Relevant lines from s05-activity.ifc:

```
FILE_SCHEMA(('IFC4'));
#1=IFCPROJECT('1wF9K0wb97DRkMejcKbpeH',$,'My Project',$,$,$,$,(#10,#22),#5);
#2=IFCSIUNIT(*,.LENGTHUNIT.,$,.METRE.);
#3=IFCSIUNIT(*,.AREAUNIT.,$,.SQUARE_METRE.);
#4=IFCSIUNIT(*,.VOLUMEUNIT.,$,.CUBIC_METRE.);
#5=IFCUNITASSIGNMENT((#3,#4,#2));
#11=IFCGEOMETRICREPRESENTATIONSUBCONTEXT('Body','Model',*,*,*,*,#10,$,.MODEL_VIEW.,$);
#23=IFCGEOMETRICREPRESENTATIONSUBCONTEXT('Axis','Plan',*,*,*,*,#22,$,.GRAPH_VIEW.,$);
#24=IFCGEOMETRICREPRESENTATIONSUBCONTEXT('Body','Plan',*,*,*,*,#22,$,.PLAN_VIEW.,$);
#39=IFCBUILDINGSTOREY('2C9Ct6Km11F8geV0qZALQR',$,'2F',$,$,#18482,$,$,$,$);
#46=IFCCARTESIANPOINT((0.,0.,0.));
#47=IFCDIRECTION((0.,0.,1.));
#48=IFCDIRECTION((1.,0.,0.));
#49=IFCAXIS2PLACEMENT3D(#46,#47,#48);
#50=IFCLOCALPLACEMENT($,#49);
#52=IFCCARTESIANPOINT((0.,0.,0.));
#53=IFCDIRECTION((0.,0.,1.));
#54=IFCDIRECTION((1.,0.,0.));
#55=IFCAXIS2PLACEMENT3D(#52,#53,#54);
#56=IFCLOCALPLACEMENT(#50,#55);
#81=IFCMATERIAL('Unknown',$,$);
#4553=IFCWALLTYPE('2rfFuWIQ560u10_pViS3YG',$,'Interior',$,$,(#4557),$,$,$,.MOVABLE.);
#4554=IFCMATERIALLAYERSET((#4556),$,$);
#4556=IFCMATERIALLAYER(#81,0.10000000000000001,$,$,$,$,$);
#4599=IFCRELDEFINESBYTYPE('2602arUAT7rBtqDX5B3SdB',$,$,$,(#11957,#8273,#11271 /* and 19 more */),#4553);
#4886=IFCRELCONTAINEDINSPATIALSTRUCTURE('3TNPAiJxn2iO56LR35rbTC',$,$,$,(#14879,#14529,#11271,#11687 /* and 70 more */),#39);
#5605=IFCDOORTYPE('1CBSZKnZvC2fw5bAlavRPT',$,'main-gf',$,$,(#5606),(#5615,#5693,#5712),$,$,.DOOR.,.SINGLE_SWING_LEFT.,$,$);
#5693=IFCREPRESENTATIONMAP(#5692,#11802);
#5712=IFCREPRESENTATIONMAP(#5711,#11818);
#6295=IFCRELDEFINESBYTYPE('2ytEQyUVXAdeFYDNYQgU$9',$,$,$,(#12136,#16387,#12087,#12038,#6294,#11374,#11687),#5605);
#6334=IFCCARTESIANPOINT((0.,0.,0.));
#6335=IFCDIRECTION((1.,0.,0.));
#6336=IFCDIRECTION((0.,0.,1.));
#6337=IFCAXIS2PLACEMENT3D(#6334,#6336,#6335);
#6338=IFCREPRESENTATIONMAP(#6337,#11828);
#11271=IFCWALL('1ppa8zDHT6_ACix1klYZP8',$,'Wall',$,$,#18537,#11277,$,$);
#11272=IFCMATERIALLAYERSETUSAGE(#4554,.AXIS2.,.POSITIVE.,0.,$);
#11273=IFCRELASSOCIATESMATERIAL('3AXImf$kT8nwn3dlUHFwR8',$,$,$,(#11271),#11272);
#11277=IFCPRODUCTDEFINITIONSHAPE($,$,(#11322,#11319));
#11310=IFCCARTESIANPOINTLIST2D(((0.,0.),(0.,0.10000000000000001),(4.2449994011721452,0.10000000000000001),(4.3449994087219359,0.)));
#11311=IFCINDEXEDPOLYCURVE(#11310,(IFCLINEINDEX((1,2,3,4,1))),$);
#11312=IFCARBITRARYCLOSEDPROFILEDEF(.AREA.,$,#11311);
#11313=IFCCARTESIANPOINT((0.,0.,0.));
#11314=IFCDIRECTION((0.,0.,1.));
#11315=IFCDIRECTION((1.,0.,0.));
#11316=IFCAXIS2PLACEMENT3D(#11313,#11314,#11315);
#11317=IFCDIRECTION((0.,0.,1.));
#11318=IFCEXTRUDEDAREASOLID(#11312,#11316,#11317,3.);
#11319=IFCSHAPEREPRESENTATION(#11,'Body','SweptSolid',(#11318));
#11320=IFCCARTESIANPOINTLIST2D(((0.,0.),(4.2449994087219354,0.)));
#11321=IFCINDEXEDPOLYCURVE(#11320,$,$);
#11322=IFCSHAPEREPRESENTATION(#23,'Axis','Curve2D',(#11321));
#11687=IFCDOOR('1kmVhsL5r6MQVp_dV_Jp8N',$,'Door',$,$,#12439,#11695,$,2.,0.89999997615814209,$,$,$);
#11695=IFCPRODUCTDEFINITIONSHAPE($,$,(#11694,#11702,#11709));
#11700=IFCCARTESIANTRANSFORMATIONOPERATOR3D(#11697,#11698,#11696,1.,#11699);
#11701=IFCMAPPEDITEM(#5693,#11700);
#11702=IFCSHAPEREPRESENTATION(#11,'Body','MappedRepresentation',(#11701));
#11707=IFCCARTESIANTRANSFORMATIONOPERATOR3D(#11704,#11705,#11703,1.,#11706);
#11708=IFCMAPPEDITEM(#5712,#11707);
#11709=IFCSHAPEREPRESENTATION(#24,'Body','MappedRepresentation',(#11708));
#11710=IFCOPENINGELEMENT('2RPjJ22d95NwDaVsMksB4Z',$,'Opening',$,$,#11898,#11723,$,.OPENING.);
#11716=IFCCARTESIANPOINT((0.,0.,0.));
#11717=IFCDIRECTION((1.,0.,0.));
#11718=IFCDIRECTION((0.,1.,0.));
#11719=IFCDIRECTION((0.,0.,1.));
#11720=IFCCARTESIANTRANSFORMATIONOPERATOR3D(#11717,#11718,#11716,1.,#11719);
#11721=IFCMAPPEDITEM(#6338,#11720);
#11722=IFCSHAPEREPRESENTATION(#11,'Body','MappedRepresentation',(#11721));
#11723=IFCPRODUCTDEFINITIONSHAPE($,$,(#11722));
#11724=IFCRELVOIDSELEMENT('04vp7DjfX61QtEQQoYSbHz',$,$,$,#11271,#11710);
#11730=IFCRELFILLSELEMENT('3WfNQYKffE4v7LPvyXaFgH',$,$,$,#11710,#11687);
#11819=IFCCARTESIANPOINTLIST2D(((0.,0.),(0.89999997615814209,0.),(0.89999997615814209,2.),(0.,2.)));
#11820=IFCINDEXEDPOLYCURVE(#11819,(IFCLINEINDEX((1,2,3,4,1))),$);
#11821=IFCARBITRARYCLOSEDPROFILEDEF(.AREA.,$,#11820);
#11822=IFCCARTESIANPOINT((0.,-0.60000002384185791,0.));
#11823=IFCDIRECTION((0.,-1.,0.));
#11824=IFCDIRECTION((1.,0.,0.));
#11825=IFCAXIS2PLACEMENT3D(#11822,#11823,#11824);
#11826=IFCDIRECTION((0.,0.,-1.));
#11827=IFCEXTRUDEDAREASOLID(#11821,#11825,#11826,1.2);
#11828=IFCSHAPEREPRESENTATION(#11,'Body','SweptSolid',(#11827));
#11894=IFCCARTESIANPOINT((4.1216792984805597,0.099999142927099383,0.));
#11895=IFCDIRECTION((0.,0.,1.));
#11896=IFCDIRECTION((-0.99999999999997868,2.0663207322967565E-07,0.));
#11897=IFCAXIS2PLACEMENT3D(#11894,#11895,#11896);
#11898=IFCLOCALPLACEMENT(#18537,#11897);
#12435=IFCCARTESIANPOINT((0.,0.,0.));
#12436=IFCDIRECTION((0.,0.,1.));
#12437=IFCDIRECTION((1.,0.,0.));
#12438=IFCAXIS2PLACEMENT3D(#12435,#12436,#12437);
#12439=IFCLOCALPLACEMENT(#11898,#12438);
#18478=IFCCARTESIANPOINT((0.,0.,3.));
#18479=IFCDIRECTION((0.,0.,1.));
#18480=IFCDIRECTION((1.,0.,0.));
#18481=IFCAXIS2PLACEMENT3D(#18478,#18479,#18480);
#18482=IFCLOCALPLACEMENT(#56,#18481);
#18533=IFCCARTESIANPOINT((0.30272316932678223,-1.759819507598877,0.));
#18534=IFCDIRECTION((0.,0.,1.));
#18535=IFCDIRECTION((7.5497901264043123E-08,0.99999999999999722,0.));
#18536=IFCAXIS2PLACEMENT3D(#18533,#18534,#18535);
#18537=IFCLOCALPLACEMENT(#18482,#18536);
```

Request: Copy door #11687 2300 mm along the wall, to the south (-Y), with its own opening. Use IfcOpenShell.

```python
import ifcopenshell
import ifcopenshell.api.feature
import ifcopenshell.api.geometry
import ifcopenshell.api.root
import ifcopenshell.geom
import ifcopenshell.util.element
import ifcopenshell.util.placement
import ifcopenshell.util.shape

model = ifcopenshell.open("s05-activity.ifc")
settings = ifcopenshell.geom.settings()


def volume(element):
    """Net volume in cubic metres, openings subtracted."""
    shape = ifcopenshell.geom.create_shape(settings, element)
    return ifcopenshell.util.shape.get_volume(shape.geometry)


door = model.by_id(11687)
opening = door.FillsVoids[0].RelatingOpeningElement
wall = opening.VoidsElements[0].RelatingBuildingElement
before = volume(wall)
shift = ifcopenshell.util.placement.get_local_placement(wall.ObjectPlacement)[:3, 0] * -2.3

# copy_class copies the void relationship, type, container and properties, but no geometry.
new_opening = ifcopenshell.api.root.copy_class(model, product=opening)
new_opening.Representation = ifcopenshell.util.element.copy_deep(
    model, opening.Representation, exclude=["IfcGeometricRepresentationContext", "IfcRepresentationMap"]
)
new_door = ifcopenshell.api.root.copy_class(model, product=door)
new_door.Representation = ifcopenshell.util.element.copy_deep(
    model, door.Representation, exclude=["IfcGeometricRepresentationContext", "IfcRepresentationMap"]
)
ifcopenshell.api.feature.add_filling(model, opening=new_opening, element=new_door)

for old, new in ((opening, new_opening), (door, new_door)):
    matrix = ifcopenshell.util.placement.get_local_placement(old.ObjectPlacement)
    matrix[:3, 3] += shift
    ifcopenshell.api.geometry.edit_object_placement(model, product=new, matrix=matrix, is_si=False)

after = volume(wall)

print(f"wall volume {before:.3f} -> {after:.3f} m3")

model.write("s05-activity_rev.ifc")
```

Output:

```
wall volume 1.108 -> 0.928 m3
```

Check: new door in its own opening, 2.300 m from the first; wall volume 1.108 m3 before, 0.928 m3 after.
